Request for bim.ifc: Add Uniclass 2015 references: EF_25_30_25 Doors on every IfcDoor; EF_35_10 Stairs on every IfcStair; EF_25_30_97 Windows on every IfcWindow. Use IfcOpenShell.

First a look at what the model holds.

```python
import ifcopenshell

model = ifcopenshell.open("bim.ifc")
print(model.schema)
print("classifications:", [c.Name for c in model.by_type("IfcClassification")])
for ifc_class in ("IfcDoor", "IfcRoof", "IfcStair", "IfcWall", "IfcWindow"):
    print(ifc_class, len(model.by_type(ifc_class)))
```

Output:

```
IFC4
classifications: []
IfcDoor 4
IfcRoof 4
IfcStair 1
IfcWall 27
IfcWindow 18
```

```python
import ifcopenshell
import ifcopenshell.api.classification

model = ifcopenshell.open("bim.ifc")

system = ifcopenshell.api.classification.add_classification(model, classification="Uniclass 2015")

codes = {
    "IfcDoor": ("EF_25_30_25", "Doors"),
    "IfcStair": ("EF_35_10", "Stairs"),
    "IfcWindow": ("EF_25_30_97", "Windows"),
}
for ifc_class, (code, name) in codes.items():
    products = model.by_type(ifc_class)
    ifcopenshell.api.classification.add_reference(
        model, products=products, classification=system, identification=code, name=name
    )
    print(code, len(products))

model.write("bim_rev.ifc")
```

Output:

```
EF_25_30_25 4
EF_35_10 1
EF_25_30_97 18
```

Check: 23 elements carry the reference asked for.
